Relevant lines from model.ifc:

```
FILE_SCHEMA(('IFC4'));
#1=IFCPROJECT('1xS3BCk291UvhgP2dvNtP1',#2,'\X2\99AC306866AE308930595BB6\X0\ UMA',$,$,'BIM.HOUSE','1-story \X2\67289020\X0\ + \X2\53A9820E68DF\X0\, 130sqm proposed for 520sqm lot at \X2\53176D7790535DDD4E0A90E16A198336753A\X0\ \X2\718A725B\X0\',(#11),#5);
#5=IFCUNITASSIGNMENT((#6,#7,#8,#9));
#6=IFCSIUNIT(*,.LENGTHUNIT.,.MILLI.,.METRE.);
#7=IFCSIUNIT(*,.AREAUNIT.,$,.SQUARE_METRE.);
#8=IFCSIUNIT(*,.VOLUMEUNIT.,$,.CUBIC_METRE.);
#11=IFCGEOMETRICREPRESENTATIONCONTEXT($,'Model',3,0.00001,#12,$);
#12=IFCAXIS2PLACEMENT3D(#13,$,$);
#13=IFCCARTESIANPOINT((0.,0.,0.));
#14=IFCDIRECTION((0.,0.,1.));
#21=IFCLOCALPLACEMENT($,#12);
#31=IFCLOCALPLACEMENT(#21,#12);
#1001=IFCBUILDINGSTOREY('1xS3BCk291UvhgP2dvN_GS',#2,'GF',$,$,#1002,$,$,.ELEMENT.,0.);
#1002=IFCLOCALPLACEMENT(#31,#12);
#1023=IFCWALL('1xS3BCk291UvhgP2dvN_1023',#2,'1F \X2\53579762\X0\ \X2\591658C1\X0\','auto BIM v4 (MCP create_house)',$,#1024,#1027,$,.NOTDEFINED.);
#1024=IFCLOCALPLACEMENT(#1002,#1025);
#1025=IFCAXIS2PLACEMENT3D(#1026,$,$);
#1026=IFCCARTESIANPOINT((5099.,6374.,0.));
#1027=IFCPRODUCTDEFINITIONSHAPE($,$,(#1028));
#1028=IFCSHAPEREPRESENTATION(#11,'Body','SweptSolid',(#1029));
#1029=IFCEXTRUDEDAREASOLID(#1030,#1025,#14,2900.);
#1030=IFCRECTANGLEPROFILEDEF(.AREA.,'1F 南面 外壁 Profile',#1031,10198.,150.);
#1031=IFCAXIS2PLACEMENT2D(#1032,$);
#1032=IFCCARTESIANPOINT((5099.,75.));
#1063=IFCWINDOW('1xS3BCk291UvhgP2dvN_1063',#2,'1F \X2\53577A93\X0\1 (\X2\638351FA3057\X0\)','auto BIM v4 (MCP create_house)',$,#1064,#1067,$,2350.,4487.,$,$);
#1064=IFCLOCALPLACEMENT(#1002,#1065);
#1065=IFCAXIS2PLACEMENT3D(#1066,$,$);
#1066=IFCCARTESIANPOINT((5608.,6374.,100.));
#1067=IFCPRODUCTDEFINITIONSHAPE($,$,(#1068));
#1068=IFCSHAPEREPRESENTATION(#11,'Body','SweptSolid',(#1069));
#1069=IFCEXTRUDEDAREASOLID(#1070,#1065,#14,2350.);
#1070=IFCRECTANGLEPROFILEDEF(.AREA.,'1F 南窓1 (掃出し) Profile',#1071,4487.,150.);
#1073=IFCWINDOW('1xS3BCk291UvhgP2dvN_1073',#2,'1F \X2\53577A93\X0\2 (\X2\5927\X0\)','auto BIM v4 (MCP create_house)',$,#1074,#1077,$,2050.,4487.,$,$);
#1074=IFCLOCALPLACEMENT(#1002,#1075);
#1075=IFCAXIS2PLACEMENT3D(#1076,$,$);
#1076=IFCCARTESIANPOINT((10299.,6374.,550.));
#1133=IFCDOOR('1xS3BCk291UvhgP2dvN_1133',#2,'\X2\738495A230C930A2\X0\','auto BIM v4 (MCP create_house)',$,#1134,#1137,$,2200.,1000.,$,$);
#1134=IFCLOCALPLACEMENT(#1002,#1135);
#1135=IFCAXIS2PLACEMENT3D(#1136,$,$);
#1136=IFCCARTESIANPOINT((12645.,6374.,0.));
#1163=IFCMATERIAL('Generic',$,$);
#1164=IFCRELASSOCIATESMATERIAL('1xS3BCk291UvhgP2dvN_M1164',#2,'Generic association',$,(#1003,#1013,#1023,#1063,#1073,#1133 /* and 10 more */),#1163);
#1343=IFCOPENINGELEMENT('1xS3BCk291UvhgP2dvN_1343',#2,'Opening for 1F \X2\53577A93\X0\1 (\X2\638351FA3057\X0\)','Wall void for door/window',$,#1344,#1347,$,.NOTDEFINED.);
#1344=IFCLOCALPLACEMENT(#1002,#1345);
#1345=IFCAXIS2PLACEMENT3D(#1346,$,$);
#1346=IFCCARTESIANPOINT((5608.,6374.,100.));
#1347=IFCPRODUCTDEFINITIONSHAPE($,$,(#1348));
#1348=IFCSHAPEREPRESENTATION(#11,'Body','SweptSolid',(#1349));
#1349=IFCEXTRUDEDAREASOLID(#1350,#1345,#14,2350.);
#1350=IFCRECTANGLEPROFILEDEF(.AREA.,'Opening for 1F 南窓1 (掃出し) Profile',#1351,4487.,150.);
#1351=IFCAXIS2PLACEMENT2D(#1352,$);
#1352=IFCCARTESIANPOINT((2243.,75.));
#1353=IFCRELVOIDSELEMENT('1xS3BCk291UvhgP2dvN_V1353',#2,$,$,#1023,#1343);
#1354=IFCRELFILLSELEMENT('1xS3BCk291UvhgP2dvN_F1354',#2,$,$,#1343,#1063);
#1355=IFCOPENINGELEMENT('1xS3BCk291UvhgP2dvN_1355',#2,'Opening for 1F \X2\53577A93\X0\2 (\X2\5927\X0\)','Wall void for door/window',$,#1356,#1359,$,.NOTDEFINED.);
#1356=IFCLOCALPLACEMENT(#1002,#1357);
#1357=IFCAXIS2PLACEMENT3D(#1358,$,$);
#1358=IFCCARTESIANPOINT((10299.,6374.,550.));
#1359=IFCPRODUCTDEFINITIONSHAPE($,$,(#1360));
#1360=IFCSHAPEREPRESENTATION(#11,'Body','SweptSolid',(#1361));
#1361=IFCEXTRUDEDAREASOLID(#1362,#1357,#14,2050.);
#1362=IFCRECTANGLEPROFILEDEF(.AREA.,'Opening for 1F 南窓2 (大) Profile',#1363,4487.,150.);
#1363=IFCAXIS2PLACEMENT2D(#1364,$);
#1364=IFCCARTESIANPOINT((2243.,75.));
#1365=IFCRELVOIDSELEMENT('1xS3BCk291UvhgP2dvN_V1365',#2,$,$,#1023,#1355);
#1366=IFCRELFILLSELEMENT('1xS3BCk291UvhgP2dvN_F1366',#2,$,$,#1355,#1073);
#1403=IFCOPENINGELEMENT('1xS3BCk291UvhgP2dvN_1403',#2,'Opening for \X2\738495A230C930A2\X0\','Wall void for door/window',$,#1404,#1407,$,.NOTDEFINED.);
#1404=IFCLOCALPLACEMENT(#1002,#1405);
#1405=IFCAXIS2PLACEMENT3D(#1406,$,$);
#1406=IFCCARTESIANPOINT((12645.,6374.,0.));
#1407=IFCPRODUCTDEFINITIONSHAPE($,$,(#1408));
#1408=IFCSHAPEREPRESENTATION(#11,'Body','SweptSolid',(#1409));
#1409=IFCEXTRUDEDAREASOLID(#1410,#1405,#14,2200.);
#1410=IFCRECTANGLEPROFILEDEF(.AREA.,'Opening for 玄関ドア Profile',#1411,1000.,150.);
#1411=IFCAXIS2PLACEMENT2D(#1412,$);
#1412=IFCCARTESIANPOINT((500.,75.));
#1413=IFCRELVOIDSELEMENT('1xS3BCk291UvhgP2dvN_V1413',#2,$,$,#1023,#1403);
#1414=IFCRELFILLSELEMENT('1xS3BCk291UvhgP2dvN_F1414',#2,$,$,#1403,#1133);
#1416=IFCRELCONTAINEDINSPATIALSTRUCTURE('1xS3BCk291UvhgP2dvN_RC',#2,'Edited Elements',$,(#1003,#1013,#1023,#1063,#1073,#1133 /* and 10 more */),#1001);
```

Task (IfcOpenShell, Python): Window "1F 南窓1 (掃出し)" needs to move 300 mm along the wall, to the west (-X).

```python
import ifcopenshell
import ifcopenshell.api.geometry
import ifcopenshell.util.placement

model = ifcopenshell.open("model.ifc")

window = model.by_guid("1xS3BCk291UvhgP2dvN_1063")
opening = window.FillsVoids[0].RelatingOpeningElement
wall = opening.VoidsElements[0].RelatingBuildingElement

wall_matrix = ifcopenshell.util.placement.get_local_placement(wall.ObjectPlacement)
shift = wall_matrix[:3, 0] * -300.0
before = ifcopenshell.util.placement.get_local_placement(window.ObjectPlacement)[:3, 3].copy()

# The window is not placed relative to its opening, so move both.
for product in (opening, window):
    matrix = ifcopenshell.util.placement.get_local_placement(product.ObjectPlacement)
    matrix[:3, 3] += shift
    ifcopenshell.api.geometry.edit_object_placement(model, product=product, matrix=matrix, is_si=False)

after = ifcopenshell.util.placement.get_local_placement(window.ObjectPlacement)[:3, 3]
print("window moved by", (after - before).round(3) + 0.0)

model.write("model_rev.ifc")
```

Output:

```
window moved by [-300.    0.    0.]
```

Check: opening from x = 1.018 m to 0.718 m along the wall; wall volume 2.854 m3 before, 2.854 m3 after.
